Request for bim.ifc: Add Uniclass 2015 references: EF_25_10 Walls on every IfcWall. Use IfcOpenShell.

First a look at what the model holds.

```python
import ifcopenshell

model = ifcopenshell.open("bim.ifc")
print(model.schema)
print("classifications:", [c.Name for c in model.by_type("IfcClassification")])
for ifc_class in ("IfcDoor", "IfcRoof", "IfcStair", "IfcWall", "IfcWindow"):
    print(ifc_class, len(model.by_type(ifc_class)))
```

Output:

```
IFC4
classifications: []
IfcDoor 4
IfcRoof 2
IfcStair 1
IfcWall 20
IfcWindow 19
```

```python
import ifcopenshell
import ifcopenshell.api.classification

model = ifcopenshell.open("bim.ifc")

system = ifcopenshell.api.classification.add_classification(model, classification="Uniclass 2015")

codes = {
    "IfcWall": ("EF_25_10", "Walls"),
}
for ifc_class, (code, name) in codes.items():
    products = model.by_type(ifc_class)
    ifcopenshell.api.classification.add_reference(
        model, products=products, classification=system, identification=code, name=name
    )
    print(code, len(products))

model.write("bim_edited.ifc")
```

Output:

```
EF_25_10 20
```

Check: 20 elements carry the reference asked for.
